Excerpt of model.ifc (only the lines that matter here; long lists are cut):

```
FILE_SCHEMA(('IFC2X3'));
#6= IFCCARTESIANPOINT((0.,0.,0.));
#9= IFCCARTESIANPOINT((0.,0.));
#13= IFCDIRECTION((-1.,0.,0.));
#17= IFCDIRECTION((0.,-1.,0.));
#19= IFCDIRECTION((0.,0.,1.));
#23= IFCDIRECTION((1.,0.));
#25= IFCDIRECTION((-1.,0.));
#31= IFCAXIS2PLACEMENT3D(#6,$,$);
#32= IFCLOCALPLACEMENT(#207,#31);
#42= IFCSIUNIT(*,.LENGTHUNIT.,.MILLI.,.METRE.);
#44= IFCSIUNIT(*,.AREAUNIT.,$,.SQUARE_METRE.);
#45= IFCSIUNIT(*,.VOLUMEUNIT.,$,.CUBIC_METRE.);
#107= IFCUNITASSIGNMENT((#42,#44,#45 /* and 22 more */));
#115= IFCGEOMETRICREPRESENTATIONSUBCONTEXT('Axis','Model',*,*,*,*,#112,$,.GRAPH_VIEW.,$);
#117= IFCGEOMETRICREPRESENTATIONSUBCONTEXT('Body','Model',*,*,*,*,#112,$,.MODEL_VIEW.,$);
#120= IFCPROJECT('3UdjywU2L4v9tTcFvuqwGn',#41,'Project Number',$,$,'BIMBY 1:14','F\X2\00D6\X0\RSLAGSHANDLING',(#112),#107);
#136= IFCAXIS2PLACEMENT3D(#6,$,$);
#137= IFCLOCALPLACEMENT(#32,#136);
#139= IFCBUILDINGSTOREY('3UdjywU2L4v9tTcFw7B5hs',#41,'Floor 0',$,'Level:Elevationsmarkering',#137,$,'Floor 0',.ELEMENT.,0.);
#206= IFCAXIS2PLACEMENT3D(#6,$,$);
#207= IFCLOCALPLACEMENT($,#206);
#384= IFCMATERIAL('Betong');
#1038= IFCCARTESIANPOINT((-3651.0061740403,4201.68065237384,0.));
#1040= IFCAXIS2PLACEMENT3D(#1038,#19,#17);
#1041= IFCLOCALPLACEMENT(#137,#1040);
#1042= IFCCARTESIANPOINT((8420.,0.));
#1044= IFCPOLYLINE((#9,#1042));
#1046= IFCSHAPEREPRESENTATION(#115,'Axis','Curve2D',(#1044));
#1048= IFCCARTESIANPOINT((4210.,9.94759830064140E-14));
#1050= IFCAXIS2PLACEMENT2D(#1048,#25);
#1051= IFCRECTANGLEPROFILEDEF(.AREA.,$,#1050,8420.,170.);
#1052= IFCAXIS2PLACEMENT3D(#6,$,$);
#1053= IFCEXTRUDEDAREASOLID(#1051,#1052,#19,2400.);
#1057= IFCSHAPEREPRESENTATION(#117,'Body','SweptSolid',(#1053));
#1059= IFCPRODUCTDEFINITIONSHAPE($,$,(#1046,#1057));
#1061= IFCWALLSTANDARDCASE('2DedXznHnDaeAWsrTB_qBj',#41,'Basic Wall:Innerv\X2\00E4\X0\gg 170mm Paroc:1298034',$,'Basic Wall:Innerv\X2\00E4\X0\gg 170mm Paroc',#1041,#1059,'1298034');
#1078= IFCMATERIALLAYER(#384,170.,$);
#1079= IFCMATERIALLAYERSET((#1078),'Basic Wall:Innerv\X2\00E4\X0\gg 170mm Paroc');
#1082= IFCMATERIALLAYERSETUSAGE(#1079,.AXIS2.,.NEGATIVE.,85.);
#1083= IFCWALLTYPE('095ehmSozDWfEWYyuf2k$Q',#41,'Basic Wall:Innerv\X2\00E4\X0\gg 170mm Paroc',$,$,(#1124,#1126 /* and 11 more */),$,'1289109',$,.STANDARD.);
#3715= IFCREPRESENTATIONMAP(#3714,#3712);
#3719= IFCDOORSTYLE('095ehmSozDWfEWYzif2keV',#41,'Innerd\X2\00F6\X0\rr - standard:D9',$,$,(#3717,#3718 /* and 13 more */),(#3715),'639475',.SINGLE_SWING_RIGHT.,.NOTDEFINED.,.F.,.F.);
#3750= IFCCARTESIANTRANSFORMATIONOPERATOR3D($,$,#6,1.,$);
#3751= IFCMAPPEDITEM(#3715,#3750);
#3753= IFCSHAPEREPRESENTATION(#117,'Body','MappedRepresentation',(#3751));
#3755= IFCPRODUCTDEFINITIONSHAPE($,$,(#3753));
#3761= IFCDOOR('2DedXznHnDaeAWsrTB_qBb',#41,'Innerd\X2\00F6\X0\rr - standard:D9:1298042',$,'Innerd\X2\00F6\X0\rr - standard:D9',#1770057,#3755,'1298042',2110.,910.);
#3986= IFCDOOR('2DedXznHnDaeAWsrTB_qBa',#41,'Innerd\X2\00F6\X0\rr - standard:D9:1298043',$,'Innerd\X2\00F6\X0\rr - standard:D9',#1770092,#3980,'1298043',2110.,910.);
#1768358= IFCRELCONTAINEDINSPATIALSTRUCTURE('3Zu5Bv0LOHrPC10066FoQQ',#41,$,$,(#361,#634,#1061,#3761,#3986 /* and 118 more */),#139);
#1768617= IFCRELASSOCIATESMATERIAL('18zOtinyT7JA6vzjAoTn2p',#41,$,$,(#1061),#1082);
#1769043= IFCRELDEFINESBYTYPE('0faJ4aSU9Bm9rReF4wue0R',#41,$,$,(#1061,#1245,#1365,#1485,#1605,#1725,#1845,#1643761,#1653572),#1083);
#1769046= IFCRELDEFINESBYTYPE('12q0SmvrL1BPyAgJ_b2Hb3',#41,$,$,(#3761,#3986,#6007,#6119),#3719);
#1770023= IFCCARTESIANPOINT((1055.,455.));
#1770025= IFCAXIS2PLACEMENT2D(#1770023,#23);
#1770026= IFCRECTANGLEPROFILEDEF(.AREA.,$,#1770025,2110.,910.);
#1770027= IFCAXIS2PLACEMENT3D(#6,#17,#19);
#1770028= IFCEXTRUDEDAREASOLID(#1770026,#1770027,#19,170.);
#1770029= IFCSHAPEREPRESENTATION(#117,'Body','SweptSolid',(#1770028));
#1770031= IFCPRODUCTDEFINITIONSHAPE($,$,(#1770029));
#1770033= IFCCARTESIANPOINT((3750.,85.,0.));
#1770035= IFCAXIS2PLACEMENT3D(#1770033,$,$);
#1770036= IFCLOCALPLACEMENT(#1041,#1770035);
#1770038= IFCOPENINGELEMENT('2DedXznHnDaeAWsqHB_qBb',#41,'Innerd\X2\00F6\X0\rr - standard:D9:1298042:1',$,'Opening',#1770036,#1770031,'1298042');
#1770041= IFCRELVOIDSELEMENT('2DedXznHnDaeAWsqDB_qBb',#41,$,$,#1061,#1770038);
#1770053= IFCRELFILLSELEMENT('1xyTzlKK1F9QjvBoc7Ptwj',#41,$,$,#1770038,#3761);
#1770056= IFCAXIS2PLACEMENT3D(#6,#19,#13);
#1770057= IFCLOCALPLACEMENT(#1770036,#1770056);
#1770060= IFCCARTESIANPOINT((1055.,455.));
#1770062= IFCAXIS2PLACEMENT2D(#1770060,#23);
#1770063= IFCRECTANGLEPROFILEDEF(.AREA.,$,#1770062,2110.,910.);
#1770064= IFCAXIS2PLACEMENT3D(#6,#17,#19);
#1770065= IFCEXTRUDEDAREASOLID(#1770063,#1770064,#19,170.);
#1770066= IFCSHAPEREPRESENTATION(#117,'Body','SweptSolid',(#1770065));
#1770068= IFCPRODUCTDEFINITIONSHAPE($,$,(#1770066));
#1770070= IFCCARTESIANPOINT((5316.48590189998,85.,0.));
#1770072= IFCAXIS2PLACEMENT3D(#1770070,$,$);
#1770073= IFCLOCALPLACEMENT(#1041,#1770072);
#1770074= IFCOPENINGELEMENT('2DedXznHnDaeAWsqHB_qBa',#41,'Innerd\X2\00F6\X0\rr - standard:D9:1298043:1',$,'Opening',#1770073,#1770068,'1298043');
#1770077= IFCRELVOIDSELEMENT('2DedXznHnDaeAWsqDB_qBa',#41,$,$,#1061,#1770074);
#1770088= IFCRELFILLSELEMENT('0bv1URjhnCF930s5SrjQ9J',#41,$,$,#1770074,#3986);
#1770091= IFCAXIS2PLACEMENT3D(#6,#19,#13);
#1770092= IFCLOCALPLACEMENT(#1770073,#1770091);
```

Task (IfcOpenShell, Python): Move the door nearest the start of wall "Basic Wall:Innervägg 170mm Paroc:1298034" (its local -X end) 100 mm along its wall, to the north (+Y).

```python
import ifcopenshell
import ifcopenshell.api.geometry
import ifcopenshell.util.placement
import ifcopenshell.util.unit

model = ifcopenshell.open("model.ifc")
unit_scale = ifcopenshell.util.unit.calculate_unit_scale(model)

door = model.by_guid("2DedXznHnDaeAWsrTB_qBb")
opening = door.FillsVoids[0].RelatingOpeningElement
wall = opening.VoidsElements[0].RelatingBuildingElement

wall_matrix = ifcopenshell.util.placement.get_local_placement(wall.ObjectPlacement)
shift = wall_matrix[:3, 0] * -0.1 / unit_scale
before = ifcopenshell.util.placement.get_local_placement(door.ObjectPlacement)[:3, 3].copy()

# The door is placed relative to its opening, so it follows when the opening moves.
matrix = ifcopenshell.util.placement.get_local_placement(opening.ObjectPlacement)
matrix[:3, 3] += shift
ifcopenshell.api.geometry.edit_object_placement(
    model, product=opening, matrix=matrix, is_si=False, should_transform_children=True
)

after = ifcopenshell.util.placement.get_local_placement(door.ObjectPlacement)[:3, 3]
print("door moved by", (after - before).round(3) + 0.0)

model.write("model-out.ifc")
```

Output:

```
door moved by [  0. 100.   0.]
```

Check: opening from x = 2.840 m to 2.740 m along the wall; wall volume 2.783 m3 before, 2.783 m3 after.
